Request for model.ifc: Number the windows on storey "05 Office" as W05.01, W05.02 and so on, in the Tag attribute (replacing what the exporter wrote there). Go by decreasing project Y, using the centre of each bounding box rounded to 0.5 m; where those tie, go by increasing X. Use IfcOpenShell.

First a look at what the model holds.

```python
import ifcopenshell
import ifcopenshell.util.element
import ifcopenshell.util.placement

model = ifcopenshell.open("model.ifc")
print(model.schema)
storey = next(s for s in model.by_type("IfcBuildingStorey") if s.Name == "05 Office")
windows = [e for e in ifcopenshell.util.element.get_decomposition(storey) if e.is_a("IfcWindow")]
for e in sorted(windows, key=lambda e: e.id()):
    origin = ifcopenshell.util.placement.get_local_placement(e.ObjectPlacement)[:3, 3]
    print(e.id(), e.Tag, e.Name, origin.round(2) + 0.0, sep=" | ")
```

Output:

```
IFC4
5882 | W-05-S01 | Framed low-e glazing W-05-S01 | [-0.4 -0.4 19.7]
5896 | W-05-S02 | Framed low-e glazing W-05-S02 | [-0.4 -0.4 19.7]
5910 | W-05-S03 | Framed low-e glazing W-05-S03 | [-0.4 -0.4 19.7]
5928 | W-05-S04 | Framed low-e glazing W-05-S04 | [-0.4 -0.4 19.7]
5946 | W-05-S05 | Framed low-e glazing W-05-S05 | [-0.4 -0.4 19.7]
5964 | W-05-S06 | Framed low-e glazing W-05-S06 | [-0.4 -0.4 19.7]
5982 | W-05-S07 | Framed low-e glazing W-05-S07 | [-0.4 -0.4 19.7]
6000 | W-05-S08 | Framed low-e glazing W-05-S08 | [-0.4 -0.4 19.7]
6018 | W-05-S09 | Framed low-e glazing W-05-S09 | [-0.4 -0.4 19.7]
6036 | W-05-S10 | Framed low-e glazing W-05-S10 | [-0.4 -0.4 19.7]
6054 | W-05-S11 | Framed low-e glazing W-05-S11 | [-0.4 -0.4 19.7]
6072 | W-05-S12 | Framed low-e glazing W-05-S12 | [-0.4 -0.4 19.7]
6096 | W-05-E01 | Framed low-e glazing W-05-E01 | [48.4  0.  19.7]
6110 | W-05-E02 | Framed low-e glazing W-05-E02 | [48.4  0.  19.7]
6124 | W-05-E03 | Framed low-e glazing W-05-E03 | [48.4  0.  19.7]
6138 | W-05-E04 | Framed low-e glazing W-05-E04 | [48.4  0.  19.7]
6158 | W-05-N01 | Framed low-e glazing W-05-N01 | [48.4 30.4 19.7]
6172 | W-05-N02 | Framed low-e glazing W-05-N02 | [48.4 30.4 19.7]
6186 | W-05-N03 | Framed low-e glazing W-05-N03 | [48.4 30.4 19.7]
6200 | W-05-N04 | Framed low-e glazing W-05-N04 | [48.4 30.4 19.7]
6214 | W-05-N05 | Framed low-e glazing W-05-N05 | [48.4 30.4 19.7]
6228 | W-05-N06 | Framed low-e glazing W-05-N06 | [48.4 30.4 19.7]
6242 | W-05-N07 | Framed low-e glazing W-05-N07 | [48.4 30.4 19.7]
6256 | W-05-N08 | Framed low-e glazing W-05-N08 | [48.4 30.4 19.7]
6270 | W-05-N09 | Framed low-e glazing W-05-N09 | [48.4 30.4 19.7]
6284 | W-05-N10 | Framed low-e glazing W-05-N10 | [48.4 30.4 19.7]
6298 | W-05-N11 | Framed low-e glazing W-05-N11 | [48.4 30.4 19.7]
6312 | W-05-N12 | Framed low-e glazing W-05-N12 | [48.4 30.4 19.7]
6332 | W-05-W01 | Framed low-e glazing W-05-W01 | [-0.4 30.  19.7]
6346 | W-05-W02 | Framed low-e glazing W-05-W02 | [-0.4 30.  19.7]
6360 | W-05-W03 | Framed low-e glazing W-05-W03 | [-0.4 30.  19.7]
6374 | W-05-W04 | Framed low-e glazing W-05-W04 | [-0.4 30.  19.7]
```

```python
import ifcopenshell
import ifcopenshell.geom
import ifcopenshell.util.element
import ifcopenshell.util.shape

model = ifcopenshell.open("model.ifc")
settings = ifcopenshell.geom.settings()
settings.set("use-world-coords", True)


def centre(element):
    shape = ifcopenshell.geom.create_shape(settings, element)
    return ifcopenshell.util.shape.get_bbox_centroid(shape.geometry)


storey = next(s for s in model.by_type("IfcBuildingStorey") if s.Name == "05 Office")
windows = [e for e in ifcopenshell.util.element.get_decomposition(storey) if e.is_a("IfcWindow")]

# Insertion points can sit at a corner or the storey origin, so sort by the geometry (in metres).
centres = {e: centre(e) for e in windows}
windows.sort(key=lambda e: (-round(centres[e][1] / 0.5), centres[e][0]))

for i, e in enumerate(windows, start=1):
    number = f"W05.{i:02d}"
    e.Tag = number
    print(e.id(), number)

model.write("model_rev.ifc")
```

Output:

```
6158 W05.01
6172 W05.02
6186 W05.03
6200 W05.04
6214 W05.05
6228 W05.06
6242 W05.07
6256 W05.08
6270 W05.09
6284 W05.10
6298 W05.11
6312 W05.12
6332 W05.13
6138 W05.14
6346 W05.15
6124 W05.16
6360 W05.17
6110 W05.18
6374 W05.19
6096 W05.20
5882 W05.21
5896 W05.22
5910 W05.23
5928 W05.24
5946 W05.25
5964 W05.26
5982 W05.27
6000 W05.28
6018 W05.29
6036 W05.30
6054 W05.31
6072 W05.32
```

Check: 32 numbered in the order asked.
